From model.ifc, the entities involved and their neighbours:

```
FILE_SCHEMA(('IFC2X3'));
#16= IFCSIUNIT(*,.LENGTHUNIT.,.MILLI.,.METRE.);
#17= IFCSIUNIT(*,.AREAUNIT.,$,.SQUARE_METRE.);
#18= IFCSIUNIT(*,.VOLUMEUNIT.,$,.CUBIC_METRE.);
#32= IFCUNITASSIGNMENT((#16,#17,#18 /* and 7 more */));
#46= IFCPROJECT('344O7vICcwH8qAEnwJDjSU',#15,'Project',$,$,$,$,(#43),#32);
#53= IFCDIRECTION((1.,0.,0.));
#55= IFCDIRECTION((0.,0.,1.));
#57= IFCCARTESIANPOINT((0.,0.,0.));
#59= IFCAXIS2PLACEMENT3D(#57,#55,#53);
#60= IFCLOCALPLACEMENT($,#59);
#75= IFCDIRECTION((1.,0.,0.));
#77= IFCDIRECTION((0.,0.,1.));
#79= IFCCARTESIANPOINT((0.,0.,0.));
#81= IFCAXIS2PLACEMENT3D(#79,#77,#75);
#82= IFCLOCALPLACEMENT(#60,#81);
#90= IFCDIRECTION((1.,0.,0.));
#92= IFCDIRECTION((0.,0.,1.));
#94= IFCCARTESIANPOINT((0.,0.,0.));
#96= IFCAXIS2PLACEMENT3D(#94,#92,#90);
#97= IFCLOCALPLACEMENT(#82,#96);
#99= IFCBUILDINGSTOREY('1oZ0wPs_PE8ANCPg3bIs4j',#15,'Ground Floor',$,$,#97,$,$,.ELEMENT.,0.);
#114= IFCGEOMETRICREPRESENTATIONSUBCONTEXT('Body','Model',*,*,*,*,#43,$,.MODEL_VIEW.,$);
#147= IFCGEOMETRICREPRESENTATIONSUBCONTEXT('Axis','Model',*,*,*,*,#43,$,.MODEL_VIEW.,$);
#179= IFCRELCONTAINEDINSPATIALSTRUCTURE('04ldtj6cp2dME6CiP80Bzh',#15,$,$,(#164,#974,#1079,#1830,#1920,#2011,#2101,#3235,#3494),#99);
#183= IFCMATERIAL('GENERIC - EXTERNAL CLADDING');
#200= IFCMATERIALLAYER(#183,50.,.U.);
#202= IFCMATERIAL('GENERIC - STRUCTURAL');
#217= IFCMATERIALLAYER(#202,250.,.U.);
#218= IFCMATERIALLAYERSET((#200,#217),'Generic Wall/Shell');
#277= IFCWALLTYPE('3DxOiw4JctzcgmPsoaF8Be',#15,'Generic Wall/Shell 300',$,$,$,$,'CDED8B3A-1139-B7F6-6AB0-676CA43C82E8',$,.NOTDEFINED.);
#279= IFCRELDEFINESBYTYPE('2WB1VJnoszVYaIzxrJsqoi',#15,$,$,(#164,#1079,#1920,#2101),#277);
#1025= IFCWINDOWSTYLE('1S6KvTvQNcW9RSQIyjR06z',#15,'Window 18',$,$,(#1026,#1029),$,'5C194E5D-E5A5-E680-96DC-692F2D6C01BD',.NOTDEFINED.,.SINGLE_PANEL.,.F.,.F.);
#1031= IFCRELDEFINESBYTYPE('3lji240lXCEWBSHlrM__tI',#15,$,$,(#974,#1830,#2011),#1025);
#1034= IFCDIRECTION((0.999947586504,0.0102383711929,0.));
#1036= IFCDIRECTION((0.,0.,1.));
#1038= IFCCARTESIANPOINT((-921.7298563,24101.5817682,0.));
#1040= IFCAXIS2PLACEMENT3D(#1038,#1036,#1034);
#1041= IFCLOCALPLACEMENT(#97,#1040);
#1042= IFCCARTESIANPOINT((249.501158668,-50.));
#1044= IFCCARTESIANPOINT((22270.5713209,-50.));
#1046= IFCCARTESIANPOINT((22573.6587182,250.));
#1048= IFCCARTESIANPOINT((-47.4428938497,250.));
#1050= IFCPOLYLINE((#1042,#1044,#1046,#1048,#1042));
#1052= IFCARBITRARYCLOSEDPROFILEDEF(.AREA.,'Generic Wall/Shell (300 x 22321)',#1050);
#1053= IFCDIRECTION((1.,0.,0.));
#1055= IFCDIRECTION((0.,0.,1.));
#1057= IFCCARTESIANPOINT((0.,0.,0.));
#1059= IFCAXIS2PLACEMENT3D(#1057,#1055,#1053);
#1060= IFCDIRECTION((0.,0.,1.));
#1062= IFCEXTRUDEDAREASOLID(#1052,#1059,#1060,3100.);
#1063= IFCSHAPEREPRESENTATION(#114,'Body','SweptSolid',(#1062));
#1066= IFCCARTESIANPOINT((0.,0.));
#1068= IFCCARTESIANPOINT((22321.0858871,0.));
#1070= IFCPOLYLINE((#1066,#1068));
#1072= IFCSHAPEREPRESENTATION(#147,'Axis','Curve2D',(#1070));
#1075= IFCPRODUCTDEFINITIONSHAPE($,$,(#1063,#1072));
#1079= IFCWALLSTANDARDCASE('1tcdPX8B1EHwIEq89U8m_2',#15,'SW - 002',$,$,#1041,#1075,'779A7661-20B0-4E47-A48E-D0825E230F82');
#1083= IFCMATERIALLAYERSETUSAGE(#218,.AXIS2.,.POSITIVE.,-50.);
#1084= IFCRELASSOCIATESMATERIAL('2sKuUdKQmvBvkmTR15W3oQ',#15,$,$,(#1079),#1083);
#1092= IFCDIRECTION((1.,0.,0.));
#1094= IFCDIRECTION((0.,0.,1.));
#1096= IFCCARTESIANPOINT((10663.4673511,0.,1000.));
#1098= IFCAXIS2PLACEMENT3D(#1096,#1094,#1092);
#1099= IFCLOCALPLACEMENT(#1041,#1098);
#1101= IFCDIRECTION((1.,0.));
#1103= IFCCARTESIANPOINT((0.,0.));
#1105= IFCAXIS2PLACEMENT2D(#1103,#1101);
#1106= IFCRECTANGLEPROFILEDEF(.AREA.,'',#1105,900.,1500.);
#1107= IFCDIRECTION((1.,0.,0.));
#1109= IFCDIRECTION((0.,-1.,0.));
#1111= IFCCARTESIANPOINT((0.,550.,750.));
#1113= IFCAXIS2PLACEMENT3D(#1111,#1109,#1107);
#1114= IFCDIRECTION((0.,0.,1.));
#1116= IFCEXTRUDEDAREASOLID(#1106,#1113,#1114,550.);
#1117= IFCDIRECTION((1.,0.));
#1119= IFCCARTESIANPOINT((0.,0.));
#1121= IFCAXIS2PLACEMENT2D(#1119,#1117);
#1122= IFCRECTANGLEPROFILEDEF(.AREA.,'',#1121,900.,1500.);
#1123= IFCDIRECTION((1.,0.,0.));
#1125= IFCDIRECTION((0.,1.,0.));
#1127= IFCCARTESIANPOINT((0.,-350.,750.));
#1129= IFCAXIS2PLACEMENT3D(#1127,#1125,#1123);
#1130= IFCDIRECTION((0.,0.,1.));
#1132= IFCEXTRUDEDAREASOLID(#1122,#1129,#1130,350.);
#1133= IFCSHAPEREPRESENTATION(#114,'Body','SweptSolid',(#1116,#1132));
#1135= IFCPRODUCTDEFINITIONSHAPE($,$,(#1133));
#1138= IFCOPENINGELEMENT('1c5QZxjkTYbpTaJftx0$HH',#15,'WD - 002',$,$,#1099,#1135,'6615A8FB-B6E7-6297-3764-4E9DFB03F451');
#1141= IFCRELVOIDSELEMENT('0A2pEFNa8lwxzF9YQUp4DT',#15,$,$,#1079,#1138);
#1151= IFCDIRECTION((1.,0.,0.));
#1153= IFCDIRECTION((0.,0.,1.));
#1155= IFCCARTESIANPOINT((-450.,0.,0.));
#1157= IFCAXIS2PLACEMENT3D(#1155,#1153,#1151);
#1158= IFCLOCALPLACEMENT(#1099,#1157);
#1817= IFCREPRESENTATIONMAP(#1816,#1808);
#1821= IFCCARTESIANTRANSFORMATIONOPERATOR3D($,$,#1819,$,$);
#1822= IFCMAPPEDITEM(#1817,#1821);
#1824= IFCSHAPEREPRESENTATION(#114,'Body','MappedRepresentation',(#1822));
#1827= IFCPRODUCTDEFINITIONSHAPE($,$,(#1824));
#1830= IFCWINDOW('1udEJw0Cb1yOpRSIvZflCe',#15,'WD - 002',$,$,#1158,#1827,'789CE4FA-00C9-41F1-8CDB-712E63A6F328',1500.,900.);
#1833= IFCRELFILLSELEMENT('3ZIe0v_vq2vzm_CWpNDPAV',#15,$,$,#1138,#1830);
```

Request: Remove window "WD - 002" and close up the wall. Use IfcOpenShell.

```python
import ifcopenshell
import ifcopenshell.api.feature
import ifcopenshell.api.root
import ifcopenshell.geom
import ifcopenshell.util.shape

model = ifcopenshell.open("model.ifc")
settings = ifcopenshell.geom.settings()


def volume(element):
    """Net volume in cubic metres, openings subtracted."""
    shape = ifcopenshell.geom.create_shape(settings, element)
    return ifcopenshell.util.shape.get_volume(shape.geometry)


window = model.by_id(1830)
opening = window.FillsVoids[0].RelatingOpeningElement
wall = opening.VoidsElements[0].RelatingBuildingElement
before = volume(wall)

ifcopenshell.api.root.remove_product(model, product=window)
ifcopenshell.api.feature.remove_feature(model, feature=opening)

after = volume(wall)

print(f"wall volume {before:.3f} -> {after:.3f} m3")

model.write("model_edited.ifc")
```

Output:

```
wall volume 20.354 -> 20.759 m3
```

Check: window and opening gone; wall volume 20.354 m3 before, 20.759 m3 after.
